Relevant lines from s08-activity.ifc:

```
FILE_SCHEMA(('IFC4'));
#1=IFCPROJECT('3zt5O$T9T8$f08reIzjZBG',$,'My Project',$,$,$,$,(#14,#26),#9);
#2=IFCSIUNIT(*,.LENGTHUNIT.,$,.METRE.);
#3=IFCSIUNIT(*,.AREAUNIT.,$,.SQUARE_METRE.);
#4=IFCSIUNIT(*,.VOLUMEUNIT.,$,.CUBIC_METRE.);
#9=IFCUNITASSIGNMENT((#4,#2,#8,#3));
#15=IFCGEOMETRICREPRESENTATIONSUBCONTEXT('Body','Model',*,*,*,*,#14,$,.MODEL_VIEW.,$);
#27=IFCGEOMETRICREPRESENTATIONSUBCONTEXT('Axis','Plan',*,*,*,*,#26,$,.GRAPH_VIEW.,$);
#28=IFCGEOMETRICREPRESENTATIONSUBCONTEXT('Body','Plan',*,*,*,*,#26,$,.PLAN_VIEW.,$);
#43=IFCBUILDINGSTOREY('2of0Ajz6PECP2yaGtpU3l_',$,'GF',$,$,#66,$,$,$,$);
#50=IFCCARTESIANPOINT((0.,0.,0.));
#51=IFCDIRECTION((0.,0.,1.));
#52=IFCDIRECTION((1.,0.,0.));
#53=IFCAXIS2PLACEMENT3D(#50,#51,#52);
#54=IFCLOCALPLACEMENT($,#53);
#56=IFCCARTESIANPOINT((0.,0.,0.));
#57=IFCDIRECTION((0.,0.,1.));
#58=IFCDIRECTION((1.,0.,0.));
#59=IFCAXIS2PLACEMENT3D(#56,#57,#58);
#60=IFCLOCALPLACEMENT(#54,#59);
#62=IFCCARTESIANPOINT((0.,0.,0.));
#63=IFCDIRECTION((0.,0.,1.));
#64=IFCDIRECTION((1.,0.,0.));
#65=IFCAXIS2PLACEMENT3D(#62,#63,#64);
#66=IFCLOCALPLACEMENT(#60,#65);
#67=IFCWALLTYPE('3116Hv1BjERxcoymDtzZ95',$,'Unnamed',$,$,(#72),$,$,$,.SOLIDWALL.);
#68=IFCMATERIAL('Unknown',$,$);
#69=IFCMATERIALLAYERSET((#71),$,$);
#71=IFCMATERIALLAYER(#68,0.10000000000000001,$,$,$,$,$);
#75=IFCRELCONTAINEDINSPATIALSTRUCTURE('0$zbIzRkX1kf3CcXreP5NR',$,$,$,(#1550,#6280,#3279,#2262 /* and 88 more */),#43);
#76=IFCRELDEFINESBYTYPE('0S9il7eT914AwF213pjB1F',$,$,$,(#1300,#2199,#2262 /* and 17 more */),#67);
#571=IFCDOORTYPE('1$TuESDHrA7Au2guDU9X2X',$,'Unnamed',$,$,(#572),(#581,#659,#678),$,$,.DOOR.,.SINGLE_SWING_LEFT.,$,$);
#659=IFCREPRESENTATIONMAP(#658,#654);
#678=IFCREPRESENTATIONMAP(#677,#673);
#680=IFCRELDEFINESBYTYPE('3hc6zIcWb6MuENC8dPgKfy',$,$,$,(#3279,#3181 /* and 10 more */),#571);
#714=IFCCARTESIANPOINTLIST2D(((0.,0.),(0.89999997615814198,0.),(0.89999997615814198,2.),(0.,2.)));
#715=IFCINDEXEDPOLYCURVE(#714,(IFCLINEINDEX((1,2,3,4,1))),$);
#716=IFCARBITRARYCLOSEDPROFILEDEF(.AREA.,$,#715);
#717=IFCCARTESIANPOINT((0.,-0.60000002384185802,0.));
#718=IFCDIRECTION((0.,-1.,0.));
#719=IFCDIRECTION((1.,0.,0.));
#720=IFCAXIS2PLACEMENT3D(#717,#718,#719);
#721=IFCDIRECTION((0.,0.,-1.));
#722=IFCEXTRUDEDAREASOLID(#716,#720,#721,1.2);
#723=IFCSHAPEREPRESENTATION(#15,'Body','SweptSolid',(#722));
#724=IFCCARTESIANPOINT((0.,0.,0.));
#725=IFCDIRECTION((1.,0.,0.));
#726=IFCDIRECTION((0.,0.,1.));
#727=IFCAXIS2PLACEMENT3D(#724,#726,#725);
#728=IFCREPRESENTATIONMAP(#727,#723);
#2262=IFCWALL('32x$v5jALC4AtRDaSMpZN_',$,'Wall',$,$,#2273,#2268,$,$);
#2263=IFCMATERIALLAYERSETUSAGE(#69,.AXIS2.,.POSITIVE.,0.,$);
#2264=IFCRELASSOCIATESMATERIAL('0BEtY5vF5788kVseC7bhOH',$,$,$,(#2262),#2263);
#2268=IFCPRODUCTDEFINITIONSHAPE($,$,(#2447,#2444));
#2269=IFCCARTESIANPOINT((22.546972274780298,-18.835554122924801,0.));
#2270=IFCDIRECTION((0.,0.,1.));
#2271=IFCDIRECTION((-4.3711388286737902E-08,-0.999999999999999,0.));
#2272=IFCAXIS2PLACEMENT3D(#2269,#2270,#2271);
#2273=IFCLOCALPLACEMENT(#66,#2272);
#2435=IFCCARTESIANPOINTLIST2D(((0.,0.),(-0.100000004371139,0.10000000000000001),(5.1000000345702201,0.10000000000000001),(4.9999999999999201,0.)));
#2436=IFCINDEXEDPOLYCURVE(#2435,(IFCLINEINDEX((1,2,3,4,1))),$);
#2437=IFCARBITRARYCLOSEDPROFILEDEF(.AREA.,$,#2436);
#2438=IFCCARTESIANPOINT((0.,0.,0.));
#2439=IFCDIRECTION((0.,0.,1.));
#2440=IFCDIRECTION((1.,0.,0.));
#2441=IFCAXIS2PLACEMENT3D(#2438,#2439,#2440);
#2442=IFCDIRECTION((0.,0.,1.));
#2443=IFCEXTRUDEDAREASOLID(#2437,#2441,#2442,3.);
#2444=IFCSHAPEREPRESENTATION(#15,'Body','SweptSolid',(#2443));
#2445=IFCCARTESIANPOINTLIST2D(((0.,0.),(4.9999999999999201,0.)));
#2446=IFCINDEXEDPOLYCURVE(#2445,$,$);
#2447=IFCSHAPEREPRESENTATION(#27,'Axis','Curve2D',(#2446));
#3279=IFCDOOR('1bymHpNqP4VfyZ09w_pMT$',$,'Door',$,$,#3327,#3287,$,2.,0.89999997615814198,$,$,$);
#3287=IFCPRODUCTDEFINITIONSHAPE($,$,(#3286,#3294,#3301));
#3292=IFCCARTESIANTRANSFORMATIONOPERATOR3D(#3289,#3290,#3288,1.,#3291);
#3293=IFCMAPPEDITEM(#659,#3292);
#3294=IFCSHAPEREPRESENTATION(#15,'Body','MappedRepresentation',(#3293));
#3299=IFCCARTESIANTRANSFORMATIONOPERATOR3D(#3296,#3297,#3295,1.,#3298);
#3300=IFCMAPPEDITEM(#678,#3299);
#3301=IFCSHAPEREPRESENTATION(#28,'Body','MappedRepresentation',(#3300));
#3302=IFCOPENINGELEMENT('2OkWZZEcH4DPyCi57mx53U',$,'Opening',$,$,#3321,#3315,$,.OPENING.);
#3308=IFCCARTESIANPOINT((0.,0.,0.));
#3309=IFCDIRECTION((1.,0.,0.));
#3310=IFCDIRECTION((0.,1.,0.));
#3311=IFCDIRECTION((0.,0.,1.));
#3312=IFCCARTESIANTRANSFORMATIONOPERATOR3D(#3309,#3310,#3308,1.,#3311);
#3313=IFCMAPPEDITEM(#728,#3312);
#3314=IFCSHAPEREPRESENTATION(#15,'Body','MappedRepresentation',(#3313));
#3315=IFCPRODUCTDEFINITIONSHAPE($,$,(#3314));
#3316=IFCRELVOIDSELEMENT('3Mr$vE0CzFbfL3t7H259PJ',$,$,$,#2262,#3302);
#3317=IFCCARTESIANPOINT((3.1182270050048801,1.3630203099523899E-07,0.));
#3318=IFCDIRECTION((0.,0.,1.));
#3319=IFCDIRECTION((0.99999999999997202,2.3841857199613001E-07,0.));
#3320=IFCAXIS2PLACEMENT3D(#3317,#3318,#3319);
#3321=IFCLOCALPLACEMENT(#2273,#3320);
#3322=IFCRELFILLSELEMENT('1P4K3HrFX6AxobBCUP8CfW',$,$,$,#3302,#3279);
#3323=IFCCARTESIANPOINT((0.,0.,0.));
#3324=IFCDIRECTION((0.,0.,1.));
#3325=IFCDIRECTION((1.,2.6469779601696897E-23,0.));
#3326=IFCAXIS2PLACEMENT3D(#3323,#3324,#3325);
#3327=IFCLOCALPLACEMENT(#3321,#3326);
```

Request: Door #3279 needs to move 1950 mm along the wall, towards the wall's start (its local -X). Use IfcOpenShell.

```python
import ifcopenshell
import ifcopenshell.api.geometry
import ifcopenshell.util.placement
import ifcopenshell.util.unit

model = ifcopenshell.open("s08-activity.ifc")
unit_scale = ifcopenshell.util.unit.calculate_unit_scale(model)

door = model.by_guid("1bymHpNqP4VfyZ09w_pMT$")
opening = door.FillsVoids[0].RelatingOpeningElement
wall = opening.VoidsElements[0].RelatingBuildingElement

wall_matrix = ifcopenshell.util.placement.get_local_placement(wall.ObjectPlacement)
shift = wall_matrix[:3, 0] * -1.95 / unit_scale
before = ifcopenshell.util.placement.get_local_placement(door.ObjectPlacement)[:3, 3].copy()

# The door is placed relative to its opening, so it follows when the opening moves.
matrix = ifcopenshell.util.placement.get_local_placement(opening.ObjectPlacement)
matrix[:3, 3] += shift
ifcopenshell.api.geometry.edit_object_placement(
    model, product=opening, matrix=matrix, is_si=False, should_transform_children=True
)

after = ifcopenshell.util.placement.get_local_placement(door.ObjectPlacement)[:3, 3]
print("door moved by", (after - before).round(3) + 0.0)

model.write("s08-activity_rev.ifc")
```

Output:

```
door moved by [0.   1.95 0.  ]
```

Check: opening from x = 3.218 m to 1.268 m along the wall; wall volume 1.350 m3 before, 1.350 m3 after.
